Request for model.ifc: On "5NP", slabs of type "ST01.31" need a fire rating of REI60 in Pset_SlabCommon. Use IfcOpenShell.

First a look at what the model holds.

```python
import ifcopenshell
import ifcopenshell.util.element

model = ifcopenshell.open("model.ifc")
print(model.schema)
storey = next(s for s in model.by_type("IfcBuildingStorey") if s.Name == "5NP")
slabs = [e for e in ifcopenshell.util.element.get_decomposition(storey) if e.is_a("IfcSlab")]
seen = {}
for e in slabs:
    element_type = ifcopenshell.util.element.get_type(e)
    key = (element_type.Name if element_type != e and element_type else None, ifcopenshell.util.element.get_pset(e, "Pset_SlabCommon", "FireRating"))
    seen[key] = seen.get(key, 0) + 1
for (name, value), count in sorted(seen.items(), key=str):
    print(count, "x", name, "|", value)
```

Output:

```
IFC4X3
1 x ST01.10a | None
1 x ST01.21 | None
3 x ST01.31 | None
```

```python
import ifcopenshell
import ifcopenshell.api.pset
import ifcopenshell.util.element

model = ifcopenshell.open("model.ifc")

storey = next(s for s in model.by_type("IfcBuildingStorey") if s.Name == "5NP")
slabs = [e for e in ifcopenshell.util.element.get_decomposition(storey) if e.is_a("IfcSlab")]

count = 0
for e in slabs:
    element_type = ifcopenshell.util.element.get_type(e)
    if element_type in (None, e) or element_type.Name != "ST01.31":
        continue
    # add_pset returns the element's existing set when there is one.
    pset = ifcopenshell.api.pset.add_pset(model, product=e, name="Pset_SlabCommon")
    ifcopenshell.api.pset.edit_pset(model, pset=pset, properties={"FireRating": "REI60"})
    count += 1

print(count, "slabs updated")

model.write("model_rev.ifc")
```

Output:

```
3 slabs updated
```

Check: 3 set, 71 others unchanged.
